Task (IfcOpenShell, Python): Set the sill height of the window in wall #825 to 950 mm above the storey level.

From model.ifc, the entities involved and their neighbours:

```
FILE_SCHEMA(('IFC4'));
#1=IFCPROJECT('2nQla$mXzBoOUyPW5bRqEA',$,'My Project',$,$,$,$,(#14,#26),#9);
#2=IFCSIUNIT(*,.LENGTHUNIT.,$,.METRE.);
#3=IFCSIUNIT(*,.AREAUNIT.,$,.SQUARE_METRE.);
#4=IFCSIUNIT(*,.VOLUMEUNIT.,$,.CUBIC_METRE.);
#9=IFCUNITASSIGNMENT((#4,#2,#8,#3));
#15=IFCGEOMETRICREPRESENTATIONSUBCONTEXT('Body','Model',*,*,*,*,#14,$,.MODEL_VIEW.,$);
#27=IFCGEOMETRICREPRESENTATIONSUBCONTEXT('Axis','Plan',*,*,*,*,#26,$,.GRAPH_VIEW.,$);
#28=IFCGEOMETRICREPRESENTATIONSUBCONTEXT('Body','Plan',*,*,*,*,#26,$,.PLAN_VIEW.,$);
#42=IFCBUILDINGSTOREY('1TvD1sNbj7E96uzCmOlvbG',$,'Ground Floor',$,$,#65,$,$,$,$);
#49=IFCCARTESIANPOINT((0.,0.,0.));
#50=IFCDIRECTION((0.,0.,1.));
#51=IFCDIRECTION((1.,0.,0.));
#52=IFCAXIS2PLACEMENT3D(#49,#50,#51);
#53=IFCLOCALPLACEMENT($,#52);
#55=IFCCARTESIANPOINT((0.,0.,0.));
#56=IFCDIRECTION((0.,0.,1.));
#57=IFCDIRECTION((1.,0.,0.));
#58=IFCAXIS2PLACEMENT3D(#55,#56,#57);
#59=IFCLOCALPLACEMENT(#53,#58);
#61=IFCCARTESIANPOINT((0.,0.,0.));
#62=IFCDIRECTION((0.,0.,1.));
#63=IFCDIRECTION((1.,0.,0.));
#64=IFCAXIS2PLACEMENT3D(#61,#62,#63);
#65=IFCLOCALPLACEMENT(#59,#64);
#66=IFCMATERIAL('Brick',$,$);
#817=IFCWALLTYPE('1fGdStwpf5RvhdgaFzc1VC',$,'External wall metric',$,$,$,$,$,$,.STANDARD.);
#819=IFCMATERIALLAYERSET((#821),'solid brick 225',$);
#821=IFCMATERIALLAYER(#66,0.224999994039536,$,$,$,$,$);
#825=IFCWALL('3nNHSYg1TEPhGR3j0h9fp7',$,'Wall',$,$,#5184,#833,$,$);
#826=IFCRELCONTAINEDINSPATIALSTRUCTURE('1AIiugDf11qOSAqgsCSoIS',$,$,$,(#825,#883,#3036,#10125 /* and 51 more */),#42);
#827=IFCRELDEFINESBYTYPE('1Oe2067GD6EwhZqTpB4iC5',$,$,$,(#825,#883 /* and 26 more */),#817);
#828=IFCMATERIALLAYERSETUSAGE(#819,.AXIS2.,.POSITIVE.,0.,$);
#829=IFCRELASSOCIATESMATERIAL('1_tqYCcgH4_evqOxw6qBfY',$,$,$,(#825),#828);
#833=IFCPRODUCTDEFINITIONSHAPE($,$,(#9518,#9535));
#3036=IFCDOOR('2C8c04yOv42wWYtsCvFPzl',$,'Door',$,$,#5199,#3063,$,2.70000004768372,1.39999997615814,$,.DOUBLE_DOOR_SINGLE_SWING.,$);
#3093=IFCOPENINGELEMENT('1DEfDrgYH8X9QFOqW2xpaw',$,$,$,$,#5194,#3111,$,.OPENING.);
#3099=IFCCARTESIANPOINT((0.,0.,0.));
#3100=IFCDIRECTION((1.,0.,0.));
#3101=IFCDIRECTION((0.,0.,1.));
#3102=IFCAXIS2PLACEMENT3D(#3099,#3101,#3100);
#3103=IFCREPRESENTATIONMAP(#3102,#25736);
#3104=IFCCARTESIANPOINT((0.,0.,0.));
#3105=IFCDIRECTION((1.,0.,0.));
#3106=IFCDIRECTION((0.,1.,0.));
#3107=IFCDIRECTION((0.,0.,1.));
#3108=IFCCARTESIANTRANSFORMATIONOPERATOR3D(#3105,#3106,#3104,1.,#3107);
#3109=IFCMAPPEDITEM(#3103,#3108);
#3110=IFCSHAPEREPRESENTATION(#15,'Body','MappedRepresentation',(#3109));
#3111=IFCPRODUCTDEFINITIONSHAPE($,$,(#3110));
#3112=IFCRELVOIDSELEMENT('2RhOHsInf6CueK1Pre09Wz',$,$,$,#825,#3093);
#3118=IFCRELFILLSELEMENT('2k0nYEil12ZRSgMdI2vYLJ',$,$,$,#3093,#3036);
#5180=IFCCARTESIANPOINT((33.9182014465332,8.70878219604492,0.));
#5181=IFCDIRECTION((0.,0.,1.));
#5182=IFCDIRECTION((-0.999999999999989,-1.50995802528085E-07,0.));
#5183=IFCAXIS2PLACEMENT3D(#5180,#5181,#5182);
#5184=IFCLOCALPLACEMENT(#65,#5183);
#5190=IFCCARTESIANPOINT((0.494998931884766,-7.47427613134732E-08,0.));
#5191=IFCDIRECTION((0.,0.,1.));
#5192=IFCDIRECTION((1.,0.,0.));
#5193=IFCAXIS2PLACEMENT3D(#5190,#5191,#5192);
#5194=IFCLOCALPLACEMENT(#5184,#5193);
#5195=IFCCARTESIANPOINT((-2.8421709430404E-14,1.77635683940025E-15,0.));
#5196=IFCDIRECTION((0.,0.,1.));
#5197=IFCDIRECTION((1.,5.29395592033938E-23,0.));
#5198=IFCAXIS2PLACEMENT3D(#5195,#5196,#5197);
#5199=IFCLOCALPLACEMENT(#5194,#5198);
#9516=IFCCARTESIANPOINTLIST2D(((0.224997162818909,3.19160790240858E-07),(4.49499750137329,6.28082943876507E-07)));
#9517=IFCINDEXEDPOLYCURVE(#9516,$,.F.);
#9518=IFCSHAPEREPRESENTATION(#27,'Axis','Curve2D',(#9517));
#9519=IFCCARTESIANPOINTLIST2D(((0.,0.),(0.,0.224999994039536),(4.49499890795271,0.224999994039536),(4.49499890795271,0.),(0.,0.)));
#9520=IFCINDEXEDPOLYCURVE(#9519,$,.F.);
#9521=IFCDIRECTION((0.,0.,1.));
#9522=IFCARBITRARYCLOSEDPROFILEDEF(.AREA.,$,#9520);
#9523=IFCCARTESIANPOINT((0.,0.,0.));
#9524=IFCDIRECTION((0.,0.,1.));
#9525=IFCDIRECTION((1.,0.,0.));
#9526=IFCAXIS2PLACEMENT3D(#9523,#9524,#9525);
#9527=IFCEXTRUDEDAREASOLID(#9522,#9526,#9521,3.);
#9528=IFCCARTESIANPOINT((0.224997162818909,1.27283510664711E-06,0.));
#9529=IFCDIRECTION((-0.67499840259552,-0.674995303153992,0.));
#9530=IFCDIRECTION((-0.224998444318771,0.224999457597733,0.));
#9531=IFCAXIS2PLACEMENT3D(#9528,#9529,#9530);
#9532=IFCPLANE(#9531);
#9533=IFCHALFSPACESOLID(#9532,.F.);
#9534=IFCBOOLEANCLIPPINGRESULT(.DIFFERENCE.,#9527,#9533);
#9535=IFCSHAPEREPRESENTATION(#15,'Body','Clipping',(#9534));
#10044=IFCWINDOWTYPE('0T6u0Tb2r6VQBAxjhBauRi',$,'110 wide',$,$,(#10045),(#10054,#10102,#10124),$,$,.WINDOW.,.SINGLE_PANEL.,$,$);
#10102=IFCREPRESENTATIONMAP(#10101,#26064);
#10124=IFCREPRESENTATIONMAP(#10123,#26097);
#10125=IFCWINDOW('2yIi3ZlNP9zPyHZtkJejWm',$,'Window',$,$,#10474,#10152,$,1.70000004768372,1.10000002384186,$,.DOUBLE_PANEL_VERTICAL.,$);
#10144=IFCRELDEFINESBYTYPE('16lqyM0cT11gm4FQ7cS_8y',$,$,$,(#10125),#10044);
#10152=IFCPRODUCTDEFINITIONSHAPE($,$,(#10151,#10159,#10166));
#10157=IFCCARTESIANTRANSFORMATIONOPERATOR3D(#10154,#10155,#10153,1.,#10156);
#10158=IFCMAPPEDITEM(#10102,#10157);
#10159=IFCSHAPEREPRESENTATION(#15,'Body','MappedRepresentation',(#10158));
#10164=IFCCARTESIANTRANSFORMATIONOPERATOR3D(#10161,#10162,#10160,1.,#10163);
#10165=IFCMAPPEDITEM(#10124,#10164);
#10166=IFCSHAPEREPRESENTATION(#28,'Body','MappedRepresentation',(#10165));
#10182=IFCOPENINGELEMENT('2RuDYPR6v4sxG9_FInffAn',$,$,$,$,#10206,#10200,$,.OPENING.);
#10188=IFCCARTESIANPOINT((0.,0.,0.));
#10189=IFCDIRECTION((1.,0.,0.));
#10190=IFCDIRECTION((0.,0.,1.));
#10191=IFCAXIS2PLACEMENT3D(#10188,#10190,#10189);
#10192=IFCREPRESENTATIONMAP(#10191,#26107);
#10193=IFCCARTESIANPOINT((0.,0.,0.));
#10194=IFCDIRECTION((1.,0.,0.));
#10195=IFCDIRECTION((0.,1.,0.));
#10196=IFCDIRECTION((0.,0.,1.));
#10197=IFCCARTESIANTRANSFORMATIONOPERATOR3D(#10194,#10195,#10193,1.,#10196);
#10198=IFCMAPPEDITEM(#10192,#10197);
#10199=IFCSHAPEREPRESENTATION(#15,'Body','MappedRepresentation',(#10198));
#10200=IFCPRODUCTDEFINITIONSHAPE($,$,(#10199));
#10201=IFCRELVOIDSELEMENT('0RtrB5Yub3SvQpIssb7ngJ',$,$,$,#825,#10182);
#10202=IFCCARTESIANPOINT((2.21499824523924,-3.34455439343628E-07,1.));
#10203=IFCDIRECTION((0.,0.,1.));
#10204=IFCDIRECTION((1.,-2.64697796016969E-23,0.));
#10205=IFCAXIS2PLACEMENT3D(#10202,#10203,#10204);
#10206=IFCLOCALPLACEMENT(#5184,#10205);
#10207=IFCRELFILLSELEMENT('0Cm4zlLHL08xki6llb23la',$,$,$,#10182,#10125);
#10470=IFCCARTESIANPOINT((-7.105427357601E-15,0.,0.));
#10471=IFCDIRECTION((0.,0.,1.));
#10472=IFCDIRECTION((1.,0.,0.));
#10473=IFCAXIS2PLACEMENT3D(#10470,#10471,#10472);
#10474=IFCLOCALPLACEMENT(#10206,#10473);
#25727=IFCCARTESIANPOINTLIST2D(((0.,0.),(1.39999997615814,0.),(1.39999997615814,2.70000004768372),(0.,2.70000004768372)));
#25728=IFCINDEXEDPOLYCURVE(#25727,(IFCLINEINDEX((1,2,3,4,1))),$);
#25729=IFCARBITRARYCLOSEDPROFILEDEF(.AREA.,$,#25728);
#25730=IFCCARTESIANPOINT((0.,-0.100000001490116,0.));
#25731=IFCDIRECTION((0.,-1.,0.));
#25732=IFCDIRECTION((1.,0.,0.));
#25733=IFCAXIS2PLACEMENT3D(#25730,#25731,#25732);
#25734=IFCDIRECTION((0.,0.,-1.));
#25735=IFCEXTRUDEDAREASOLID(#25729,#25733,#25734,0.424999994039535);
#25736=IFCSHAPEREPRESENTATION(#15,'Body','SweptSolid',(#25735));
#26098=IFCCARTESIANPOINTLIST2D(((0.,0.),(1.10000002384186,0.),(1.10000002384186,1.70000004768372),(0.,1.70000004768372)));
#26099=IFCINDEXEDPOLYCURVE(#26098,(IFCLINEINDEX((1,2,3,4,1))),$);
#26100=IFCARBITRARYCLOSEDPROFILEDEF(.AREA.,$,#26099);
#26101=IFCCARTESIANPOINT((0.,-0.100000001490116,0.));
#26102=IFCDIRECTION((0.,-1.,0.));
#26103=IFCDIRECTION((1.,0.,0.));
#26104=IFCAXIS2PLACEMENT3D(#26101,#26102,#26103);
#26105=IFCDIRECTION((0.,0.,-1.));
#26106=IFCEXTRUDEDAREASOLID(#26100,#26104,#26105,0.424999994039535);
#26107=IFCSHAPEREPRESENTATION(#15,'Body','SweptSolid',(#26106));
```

```python
import numpy as np
import ifcopenshell
import ifcopenshell.api.geometry
import ifcopenshell.geom
import ifcopenshell.util.element
import ifcopenshell.util.placement
import ifcopenshell.util.shape
import ifcopenshell.util.unit

model = ifcopenshell.open("model.ifc")
unit_scale = ifcopenshell.util.unit.calculate_unit_scale(model)

window = model.by_guid("2yIi3ZlNP9zPyHZtkJejWm")
opening = window.FillsVoids[0].RelatingOpeningElement
storey = ifcopenshell.util.element.get_container(window, ifc_class="IfcBuildingStorey")
level = ifcopenshell.util.placement.get_local_placement(storey.ObjectPlacement)[2, 3]

# The opening's origin need not be at the sill, so measure its lowest point.
shape = ifcopenshell.geom.create_shape(ifcopenshell.geom.settings(), opening)
bottom = ifcopenshell.util.shape.get_shape_bottom_elevation(shape, shape.geometry) / unit_scale
dz = level + 0.95 / unit_scale - bottom

shift = np.array([0.0, 0.0, dz])
# The window is placed relative to its opening, so it follows when the opening moves.
matrix = ifcopenshell.util.placement.get_local_placement(opening.ObjectPlacement)
matrix[:3, 3] += shift
ifcopenshell.api.geometry.edit_object_placement(
    model, product=opening, matrix=matrix, is_si=False, should_transform_children=True
)

print(f"moved by {dz * unit_scale:+.3f} m")

model.write("model_edited.ifc")
```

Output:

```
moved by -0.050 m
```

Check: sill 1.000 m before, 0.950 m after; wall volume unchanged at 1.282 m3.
